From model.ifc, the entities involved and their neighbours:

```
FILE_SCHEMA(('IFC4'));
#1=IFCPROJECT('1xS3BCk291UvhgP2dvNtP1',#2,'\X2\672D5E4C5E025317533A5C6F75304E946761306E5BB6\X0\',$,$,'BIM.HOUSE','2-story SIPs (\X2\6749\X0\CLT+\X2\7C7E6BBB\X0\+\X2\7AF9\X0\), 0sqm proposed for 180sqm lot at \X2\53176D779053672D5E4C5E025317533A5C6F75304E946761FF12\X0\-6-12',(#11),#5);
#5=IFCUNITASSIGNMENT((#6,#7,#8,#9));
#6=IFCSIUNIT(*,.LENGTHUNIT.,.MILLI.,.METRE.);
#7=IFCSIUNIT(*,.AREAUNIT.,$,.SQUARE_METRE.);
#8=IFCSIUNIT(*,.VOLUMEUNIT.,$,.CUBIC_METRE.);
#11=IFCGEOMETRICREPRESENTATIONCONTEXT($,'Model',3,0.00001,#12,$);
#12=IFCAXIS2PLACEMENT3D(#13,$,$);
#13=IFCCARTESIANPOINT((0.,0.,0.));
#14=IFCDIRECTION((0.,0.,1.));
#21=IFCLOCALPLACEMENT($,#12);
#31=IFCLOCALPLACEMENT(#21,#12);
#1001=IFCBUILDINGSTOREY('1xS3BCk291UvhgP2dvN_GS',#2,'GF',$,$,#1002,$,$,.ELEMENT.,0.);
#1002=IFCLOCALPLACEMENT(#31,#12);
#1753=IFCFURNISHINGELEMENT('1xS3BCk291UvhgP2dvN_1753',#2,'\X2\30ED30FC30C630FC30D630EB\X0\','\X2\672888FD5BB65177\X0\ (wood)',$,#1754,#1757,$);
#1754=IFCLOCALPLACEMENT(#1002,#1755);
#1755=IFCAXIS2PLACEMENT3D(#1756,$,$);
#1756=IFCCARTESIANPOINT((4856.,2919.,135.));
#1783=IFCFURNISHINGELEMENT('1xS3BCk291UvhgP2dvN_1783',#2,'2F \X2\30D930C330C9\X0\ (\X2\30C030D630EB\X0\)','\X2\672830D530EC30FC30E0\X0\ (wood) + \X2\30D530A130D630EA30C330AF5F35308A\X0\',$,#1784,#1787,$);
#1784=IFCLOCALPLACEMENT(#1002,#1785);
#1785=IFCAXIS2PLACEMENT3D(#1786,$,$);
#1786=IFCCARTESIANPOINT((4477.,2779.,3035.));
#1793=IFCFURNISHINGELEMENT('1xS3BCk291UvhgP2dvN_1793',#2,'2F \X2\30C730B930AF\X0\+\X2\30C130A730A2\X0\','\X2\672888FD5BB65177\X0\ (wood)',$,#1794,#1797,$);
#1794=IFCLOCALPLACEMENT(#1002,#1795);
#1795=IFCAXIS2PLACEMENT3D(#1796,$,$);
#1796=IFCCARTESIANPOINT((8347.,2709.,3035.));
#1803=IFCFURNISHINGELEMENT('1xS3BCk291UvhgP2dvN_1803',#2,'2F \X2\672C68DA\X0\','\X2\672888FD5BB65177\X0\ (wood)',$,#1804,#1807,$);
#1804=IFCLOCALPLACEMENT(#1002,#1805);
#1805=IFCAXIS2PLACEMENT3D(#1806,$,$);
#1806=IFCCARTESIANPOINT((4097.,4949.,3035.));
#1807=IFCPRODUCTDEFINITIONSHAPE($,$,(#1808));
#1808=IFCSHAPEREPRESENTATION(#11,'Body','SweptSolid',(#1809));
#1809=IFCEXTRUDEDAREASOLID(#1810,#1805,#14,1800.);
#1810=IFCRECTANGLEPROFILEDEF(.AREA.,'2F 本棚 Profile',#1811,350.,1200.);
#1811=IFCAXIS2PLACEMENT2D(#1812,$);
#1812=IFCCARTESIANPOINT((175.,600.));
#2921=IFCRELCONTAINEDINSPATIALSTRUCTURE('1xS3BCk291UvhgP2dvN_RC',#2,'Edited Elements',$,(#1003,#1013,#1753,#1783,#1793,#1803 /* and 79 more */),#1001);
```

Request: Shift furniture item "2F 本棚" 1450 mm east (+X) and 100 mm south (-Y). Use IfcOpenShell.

```python
import ifcopenshell
import ifcopenshell.api.geometry
import ifcopenshell.util.placement

model = ifcopenshell.open("model.ifc")

item = model.by_guid("1xS3BCk291UvhgP2dvN_1803")
matrix = ifcopenshell.util.placement.get_local_placement(item.ObjectPlacement)
matrix[0, 3] += 1450.0
matrix[1, 3] -= 100.0
ifcopenshell.api.geometry.edit_object_placement(model, product=item, matrix=matrix, is_si=False)

print(ifcopenshell.util.placement.get_local_placement(item.ObjectPlacement).round(3) + 0.0)

model.write("model_rev.ifc")
```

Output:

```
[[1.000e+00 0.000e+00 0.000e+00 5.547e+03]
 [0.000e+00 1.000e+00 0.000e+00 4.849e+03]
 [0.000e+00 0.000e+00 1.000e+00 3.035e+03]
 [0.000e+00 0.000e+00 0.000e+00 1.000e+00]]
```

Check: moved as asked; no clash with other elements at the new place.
